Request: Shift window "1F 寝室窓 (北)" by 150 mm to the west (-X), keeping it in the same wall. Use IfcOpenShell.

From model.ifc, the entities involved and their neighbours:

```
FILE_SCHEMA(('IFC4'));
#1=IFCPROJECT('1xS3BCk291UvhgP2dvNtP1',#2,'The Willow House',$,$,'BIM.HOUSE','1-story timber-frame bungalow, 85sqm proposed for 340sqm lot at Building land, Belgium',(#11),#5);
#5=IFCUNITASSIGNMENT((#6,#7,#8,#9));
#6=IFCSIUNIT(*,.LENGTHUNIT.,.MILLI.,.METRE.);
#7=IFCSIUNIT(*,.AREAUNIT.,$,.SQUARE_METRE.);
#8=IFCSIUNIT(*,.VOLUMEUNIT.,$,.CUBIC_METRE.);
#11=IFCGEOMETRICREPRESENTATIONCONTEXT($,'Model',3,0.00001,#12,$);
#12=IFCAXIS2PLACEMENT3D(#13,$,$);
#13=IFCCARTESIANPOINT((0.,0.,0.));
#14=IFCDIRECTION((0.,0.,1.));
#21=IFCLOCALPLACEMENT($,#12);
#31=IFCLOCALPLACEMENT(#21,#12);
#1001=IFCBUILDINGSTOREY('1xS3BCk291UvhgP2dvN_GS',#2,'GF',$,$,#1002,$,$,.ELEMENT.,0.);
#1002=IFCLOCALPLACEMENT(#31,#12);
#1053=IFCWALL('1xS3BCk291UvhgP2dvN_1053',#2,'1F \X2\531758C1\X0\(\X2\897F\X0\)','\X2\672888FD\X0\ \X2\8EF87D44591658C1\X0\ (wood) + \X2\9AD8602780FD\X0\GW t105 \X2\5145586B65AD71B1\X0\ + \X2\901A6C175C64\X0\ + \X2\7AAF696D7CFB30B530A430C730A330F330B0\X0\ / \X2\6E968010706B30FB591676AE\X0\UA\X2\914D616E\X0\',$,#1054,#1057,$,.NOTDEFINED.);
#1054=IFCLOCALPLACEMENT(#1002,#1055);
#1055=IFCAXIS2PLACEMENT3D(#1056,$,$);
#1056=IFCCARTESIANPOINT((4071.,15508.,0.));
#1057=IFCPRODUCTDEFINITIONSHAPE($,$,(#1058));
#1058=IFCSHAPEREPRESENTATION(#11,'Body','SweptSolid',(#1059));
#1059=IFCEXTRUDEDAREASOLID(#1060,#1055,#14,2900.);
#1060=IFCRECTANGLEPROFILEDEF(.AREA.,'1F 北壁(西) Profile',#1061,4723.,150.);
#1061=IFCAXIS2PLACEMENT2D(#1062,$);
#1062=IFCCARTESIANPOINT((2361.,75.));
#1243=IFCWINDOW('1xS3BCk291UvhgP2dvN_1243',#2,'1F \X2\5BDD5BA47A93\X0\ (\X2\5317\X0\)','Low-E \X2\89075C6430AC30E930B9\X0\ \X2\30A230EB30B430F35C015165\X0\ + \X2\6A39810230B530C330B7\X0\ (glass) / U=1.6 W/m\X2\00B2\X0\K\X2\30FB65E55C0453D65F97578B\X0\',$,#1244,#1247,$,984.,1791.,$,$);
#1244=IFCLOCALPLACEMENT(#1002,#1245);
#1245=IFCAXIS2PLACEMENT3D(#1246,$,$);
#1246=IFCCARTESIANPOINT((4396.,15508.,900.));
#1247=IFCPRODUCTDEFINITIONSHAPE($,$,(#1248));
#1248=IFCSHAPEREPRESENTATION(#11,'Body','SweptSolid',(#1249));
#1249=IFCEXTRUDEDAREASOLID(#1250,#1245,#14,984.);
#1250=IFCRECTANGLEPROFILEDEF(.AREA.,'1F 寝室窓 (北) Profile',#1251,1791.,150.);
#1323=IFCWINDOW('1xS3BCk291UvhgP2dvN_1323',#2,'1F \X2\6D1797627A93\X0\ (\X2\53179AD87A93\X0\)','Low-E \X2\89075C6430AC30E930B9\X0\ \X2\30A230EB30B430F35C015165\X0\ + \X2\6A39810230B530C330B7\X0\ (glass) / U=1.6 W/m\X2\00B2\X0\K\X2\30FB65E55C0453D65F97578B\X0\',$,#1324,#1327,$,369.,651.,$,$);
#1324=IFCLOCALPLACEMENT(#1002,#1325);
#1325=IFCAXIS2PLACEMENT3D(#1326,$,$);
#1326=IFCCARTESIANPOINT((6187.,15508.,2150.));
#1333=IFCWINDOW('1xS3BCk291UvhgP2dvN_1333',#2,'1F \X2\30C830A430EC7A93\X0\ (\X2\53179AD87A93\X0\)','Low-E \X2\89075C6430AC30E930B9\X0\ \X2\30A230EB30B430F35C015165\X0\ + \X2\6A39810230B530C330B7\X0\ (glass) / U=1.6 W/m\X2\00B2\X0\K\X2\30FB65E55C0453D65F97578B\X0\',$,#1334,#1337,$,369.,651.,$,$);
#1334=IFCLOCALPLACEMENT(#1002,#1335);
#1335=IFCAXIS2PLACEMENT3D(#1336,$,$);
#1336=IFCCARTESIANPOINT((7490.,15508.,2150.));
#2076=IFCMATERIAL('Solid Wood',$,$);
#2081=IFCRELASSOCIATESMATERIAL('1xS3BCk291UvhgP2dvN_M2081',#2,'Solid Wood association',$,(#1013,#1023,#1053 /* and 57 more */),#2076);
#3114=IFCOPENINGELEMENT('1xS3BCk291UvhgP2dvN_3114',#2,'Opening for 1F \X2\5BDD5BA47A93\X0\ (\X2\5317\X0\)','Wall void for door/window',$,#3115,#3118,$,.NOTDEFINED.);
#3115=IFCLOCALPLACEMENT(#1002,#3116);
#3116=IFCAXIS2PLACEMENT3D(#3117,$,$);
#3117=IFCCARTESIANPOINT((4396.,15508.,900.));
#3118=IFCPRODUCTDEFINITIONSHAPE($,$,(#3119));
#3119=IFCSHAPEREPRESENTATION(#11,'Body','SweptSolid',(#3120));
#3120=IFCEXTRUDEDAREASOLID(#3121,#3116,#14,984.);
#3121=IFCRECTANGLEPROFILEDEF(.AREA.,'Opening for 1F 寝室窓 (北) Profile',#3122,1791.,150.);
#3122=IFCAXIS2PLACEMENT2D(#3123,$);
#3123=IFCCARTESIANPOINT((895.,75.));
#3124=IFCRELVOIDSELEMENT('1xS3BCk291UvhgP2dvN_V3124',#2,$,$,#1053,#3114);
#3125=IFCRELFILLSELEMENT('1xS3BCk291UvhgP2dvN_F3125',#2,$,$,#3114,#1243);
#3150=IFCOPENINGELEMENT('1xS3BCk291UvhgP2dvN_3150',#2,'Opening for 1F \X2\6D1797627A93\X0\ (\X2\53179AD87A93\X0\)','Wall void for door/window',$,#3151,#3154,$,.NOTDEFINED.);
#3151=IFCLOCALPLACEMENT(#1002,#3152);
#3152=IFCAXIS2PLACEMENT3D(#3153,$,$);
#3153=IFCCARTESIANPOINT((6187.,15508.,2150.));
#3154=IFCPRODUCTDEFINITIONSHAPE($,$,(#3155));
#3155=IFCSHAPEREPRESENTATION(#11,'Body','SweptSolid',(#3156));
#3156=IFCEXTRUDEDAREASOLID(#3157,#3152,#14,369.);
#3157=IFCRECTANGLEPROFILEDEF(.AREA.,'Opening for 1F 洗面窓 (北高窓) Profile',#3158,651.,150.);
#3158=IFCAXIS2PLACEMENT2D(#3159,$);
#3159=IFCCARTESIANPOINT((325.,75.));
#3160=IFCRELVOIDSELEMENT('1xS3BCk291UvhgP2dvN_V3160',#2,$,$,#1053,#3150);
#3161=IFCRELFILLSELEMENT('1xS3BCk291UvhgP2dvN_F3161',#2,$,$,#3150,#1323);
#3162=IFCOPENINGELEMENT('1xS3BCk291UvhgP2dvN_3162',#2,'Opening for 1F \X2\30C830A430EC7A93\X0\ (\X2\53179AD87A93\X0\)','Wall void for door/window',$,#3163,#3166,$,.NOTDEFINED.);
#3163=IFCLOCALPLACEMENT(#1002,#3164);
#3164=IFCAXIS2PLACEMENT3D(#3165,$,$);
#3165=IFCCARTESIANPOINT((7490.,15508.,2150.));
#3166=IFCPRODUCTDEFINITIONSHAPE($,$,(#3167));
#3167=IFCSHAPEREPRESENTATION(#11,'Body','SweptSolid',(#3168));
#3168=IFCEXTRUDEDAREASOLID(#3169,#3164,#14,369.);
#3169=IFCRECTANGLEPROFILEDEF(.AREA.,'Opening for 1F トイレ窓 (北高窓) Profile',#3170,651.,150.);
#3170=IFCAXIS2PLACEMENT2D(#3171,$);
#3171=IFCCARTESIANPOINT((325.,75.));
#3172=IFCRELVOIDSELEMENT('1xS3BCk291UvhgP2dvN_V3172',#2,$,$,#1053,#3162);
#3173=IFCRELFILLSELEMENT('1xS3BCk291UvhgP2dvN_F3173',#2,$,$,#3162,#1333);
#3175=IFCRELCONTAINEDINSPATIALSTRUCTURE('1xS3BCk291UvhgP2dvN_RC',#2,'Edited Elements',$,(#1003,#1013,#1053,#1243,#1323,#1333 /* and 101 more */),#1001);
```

```python
import ifcopenshell
import ifcopenshell.api.geometry
import ifcopenshell.util.placement

model = ifcopenshell.open("model.ifc")

window = model.by_guid("1xS3BCk291UvhgP2dvN_1243")
opening = window.FillsVoids[0].RelatingOpeningElement
wall = opening.VoidsElements[0].RelatingBuildingElement

wall_matrix = ifcopenshell.util.placement.get_local_placement(wall.ObjectPlacement)
shift = wall_matrix[:3, 0] * -150.0
before = ifcopenshell.util.placement.get_local_placement(window.ObjectPlacement)[:3, 3].copy()

# The window is not placed relative to its opening, so move both.
for product in (opening, window):
    matrix = ifcopenshell.util.placement.get_local_placement(product.ObjectPlacement)
    matrix[:3, 3] += shift
    ifcopenshell.api.geometry.edit_object_placement(model, product=product, matrix=matrix, is_si=False)

after = ifcopenshell.util.placement.get_local_placement(window.ObjectPlacement)[:3, 3]
print("window moved by", (after - before).round(3) + 0.0)

model.write("model_edited.ifc")
```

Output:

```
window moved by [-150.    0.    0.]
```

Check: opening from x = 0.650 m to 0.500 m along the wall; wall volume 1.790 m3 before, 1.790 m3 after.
